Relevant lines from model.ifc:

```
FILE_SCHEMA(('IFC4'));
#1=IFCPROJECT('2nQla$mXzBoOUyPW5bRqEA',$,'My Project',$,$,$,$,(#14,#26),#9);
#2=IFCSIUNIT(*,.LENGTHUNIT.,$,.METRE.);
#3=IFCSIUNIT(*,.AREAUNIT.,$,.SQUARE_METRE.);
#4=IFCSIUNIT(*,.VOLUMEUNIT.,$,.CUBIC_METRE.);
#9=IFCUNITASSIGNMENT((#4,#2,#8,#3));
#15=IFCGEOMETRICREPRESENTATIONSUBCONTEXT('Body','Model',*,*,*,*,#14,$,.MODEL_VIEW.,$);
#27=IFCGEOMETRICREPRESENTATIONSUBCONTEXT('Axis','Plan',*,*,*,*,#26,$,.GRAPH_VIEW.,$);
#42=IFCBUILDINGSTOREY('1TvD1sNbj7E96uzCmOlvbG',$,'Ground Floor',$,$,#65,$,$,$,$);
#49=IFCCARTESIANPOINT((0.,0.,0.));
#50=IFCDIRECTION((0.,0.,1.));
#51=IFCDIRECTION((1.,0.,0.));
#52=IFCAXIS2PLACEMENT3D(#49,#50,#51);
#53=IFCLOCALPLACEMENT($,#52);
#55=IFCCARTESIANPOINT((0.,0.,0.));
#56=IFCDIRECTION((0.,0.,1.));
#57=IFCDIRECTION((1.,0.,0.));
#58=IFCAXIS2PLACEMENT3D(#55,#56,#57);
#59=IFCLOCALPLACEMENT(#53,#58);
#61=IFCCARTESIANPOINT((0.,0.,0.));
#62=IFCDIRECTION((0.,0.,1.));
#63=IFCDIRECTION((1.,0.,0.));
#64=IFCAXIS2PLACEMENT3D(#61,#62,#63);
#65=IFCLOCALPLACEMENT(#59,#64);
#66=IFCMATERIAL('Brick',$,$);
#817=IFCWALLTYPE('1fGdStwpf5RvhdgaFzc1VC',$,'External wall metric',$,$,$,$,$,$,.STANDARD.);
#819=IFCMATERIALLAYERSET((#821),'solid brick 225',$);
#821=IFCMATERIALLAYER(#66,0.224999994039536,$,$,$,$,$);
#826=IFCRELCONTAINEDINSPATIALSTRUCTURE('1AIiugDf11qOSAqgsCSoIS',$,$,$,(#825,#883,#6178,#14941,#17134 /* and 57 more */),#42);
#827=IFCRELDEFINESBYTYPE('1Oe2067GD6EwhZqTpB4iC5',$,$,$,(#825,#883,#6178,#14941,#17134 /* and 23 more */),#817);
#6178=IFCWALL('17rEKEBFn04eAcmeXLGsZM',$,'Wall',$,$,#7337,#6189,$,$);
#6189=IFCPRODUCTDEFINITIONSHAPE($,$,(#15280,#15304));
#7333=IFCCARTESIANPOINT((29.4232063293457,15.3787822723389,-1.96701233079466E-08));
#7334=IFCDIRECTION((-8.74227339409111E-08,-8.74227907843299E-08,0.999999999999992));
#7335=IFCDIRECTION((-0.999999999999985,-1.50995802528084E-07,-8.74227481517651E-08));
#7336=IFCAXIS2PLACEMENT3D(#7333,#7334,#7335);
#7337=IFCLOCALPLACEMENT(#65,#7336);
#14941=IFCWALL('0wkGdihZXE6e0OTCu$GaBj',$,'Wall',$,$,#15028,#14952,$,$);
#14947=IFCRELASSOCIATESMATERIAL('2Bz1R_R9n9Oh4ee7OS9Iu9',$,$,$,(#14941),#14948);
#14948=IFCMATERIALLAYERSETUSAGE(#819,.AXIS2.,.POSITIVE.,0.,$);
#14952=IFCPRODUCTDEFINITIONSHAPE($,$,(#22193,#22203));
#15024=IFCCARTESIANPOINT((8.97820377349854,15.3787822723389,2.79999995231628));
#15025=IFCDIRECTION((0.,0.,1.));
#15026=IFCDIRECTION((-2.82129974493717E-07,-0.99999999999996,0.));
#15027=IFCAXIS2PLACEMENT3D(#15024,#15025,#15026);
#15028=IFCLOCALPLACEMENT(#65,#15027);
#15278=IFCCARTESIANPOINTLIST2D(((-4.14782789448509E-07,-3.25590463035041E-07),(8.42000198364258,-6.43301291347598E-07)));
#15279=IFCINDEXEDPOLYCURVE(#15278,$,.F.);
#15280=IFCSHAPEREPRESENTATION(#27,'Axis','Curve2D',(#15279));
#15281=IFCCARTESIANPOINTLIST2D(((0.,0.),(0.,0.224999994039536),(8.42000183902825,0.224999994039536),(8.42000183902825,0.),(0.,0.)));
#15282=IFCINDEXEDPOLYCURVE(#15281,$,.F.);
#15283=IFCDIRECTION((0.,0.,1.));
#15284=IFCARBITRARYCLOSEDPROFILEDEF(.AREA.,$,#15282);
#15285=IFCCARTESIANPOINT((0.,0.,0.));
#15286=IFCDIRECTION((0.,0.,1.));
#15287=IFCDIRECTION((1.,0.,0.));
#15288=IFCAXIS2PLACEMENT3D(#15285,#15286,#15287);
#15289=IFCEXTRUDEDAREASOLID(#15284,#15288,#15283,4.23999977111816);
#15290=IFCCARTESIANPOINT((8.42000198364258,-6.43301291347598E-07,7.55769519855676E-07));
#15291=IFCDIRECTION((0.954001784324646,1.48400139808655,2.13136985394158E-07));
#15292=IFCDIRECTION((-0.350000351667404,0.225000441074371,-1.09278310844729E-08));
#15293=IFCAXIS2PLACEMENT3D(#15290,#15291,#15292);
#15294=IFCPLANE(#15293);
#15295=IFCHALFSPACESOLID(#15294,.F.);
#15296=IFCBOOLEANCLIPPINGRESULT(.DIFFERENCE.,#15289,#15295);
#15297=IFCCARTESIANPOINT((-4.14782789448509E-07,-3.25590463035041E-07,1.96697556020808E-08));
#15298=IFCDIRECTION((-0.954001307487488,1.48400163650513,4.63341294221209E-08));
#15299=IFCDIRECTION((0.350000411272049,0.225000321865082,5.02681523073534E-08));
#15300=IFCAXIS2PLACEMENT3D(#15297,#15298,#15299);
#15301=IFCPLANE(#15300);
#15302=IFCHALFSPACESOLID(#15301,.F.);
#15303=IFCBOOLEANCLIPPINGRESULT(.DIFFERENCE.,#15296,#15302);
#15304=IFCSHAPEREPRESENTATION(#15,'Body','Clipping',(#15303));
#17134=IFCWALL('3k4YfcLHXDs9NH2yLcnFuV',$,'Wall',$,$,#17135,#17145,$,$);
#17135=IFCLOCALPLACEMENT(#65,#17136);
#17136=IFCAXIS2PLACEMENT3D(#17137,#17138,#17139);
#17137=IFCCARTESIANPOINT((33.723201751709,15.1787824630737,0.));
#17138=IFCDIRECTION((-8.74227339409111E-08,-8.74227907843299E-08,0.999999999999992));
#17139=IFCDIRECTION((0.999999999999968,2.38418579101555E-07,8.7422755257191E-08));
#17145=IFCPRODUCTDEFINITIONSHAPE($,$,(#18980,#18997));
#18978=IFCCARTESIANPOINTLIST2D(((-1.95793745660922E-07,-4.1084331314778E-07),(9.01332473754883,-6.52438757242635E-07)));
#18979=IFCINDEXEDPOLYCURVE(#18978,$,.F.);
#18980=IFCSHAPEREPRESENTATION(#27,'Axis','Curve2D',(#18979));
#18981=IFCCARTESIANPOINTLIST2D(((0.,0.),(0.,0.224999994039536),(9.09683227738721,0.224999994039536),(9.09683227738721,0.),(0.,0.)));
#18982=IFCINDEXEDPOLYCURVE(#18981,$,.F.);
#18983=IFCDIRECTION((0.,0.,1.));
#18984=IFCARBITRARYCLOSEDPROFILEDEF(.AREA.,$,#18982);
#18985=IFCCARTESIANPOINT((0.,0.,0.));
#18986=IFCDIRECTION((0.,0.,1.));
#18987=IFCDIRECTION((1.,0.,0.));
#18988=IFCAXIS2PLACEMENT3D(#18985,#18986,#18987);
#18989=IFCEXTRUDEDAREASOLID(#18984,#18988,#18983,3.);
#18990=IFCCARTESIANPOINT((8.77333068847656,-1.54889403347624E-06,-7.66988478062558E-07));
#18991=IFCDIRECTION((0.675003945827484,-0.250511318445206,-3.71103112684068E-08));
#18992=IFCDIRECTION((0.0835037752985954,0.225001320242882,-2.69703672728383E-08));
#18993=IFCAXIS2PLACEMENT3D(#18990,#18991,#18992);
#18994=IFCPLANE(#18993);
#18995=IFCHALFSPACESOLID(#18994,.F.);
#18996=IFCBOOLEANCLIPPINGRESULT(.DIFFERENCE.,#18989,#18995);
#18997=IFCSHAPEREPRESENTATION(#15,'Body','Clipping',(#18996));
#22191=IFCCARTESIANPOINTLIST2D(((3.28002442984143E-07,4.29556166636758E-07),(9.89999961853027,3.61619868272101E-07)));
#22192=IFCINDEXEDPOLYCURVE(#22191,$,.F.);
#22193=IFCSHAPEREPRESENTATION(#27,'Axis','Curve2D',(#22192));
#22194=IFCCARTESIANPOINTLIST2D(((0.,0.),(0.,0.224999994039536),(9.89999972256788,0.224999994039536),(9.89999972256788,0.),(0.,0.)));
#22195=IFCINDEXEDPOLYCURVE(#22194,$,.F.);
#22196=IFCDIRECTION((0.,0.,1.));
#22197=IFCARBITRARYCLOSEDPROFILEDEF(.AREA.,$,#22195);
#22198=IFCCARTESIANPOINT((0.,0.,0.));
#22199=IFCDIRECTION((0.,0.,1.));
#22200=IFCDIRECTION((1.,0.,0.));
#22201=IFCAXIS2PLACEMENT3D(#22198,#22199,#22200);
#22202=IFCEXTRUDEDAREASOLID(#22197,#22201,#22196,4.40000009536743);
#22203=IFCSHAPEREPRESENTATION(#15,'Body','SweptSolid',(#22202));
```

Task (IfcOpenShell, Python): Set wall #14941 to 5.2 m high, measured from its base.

```python
import ifcopenshell
import ifcopenshell.geom
import ifcopenshell.util.representation
import ifcopenshell.util.shape
import ifcopenshell.util.unit

model = ifcopenshell.open("model.ifc")
unit_scale = ifcopenshell.util.unit.calculate_unit_scale(model)
settings = ifcopenshell.geom.settings()


def volume(element):
    """Net volume in cubic metres, openings subtracted."""
    shape = ifcopenshell.geom.create_shape(settings, element)
    return ifcopenshell.util.shape.get_volume(shape.geometry)


wall = model.by_guid("0wkGdihZXE6e0OTCu$GaBj")
before = volume(wall)

body = ifcopenshell.util.representation.get_representation(wall, "Model", "Body")
solid = body.Items[0]
old_height = solid.Depth
solid.Depth = 5.2 / unit_scale
after = volume(wall)

print(f"height {old_height:g} -> {solid.Depth:g}, volume {before:.3f} -> {after:.3f} m3")

model.write("model_rev.ifc")
```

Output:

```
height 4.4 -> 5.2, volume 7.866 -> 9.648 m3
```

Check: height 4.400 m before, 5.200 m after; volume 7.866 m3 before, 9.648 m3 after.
